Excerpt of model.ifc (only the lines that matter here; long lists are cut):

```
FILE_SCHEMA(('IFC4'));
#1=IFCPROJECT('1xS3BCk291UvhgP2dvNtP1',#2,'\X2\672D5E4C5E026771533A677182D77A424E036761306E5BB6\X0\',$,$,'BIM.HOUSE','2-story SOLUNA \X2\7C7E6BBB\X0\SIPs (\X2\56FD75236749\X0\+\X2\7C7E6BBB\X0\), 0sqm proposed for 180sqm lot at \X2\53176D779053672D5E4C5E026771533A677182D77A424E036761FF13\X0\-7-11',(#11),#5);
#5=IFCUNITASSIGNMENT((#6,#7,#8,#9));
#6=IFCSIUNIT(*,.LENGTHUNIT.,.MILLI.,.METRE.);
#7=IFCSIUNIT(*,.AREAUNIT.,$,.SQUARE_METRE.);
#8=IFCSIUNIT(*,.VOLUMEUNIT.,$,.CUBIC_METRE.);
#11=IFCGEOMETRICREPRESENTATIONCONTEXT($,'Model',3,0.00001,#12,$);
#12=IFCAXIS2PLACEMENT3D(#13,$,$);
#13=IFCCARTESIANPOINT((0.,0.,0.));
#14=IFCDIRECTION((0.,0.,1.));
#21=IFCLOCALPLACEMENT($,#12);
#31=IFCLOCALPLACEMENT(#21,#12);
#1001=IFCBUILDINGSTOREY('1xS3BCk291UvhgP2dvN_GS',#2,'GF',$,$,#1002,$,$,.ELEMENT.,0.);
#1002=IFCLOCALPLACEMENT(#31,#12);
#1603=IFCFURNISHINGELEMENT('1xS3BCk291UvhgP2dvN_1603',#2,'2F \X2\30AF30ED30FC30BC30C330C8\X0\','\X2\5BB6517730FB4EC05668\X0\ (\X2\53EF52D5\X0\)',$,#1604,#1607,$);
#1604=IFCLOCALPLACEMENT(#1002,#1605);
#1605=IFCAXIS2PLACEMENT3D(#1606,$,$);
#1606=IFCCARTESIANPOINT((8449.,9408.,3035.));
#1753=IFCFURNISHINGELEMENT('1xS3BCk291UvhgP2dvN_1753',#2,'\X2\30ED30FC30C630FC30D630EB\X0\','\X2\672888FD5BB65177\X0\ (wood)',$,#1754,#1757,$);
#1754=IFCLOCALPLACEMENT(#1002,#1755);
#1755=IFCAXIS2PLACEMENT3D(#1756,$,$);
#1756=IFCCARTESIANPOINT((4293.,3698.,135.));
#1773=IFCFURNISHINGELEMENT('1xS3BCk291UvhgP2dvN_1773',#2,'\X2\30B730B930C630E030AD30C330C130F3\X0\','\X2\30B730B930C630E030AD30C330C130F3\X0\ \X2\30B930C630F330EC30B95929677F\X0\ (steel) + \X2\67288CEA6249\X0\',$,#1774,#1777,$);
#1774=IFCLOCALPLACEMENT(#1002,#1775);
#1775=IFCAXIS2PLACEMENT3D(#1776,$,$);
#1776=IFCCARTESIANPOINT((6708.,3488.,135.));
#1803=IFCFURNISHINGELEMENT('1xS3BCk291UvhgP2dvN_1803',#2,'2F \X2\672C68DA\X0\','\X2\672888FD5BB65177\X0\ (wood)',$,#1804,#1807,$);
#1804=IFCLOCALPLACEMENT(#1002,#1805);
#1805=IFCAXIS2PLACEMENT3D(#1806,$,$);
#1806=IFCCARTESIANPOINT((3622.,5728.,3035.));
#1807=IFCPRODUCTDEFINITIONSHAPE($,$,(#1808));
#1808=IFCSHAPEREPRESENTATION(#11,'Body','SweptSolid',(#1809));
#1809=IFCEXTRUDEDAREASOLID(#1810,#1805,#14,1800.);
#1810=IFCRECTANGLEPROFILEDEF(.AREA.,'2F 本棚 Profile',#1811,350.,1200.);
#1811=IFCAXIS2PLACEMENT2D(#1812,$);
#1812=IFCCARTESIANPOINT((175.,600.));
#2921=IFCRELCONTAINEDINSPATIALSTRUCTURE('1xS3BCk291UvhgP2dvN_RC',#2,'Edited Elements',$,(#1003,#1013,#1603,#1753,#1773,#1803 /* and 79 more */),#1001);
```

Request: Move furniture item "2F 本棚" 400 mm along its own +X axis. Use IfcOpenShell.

```python
import ifcopenshell
import ifcopenshell.api.geometry
import ifcopenshell.util.placement

model = ifcopenshell.open("model.ifc")

item = model.by_guid("1xS3BCk291UvhgP2dvN_1803")
matrix = ifcopenshell.util.placement.get_local_placement(item.ObjectPlacement)
matrix[:3, 3] += matrix[:3, 0] * 400.0
ifcopenshell.api.geometry.edit_object_placement(model, product=item, matrix=matrix, is_si=False)

print(ifcopenshell.util.placement.get_local_placement(item.ObjectPlacement).round(3) + 0.0)

model.write("model_edited.ifc")
```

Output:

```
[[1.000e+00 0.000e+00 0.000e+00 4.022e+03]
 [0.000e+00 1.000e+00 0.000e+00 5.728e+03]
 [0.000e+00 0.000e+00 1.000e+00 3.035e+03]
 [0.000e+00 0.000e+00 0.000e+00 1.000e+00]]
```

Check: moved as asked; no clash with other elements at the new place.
